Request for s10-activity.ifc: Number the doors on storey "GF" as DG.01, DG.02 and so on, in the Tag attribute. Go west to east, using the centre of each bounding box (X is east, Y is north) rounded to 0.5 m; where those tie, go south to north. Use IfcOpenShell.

First a look at what the model holds.

```python
import ifcopenshell
import ifcopenshell.util.element
import ifcopenshell.util.placement

model = ifcopenshell.open("s10-activity.ifc")
print(model.schema)
storey = next(s for s in model.by_type("IfcBuildingStorey") if s.Name == "GF")
doors = [e for e in ifcopenshell.util.element.get_decomposition(storey) if e.is_a("IfcDoor")]
for e in sorted(doors, key=lambda e: e.id()):
    origin = ifcopenshell.util.placement.get_local_placement(e.ObjectPlacement)[:3, 3]
    print(e.id(), e.Tag, e.Name, origin.round(2) + 0.0, sep=" | ")
```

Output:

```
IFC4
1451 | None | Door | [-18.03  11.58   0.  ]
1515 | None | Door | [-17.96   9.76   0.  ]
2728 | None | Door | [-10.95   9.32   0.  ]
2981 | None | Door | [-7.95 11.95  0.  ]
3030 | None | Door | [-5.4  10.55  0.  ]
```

```python
import ifcopenshell
import ifcopenshell.geom
import ifcopenshell.util.element
import ifcopenshell.util.shape

model = ifcopenshell.open("s10-activity.ifc")
settings = ifcopenshell.geom.settings()
settings.set("use-world-coords", True)


def centre(element):
    shape = ifcopenshell.geom.create_shape(settings, element)
    return ifcopenshell.util.shape.get_bbox_centroid(shape.geometry)


storey = next(s for s in model.by_type("IfcBuildingStorey") if s.Name == "GF")
doors = [e for e in ifcopenshell.util.element.get_decomposition(storey) if e.is_a("IfcDoor")]

# Insertion points can sit at a corner or the storey origin, so sort by the geometry (in metres).
centres = {e: centre(e) for e in doors}
doors.sort(key=lambda e: (round(centres[e][0] / 0.5), centres[e][1]))

for i, e in enumerate(doors, start=1):
    number = f"DG.{i:02d}"
    e.Tag = number
    print(e.id(), number)

model.write("s10-activity_updated.ifc")
```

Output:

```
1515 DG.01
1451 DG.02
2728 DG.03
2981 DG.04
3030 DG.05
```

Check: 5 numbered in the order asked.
